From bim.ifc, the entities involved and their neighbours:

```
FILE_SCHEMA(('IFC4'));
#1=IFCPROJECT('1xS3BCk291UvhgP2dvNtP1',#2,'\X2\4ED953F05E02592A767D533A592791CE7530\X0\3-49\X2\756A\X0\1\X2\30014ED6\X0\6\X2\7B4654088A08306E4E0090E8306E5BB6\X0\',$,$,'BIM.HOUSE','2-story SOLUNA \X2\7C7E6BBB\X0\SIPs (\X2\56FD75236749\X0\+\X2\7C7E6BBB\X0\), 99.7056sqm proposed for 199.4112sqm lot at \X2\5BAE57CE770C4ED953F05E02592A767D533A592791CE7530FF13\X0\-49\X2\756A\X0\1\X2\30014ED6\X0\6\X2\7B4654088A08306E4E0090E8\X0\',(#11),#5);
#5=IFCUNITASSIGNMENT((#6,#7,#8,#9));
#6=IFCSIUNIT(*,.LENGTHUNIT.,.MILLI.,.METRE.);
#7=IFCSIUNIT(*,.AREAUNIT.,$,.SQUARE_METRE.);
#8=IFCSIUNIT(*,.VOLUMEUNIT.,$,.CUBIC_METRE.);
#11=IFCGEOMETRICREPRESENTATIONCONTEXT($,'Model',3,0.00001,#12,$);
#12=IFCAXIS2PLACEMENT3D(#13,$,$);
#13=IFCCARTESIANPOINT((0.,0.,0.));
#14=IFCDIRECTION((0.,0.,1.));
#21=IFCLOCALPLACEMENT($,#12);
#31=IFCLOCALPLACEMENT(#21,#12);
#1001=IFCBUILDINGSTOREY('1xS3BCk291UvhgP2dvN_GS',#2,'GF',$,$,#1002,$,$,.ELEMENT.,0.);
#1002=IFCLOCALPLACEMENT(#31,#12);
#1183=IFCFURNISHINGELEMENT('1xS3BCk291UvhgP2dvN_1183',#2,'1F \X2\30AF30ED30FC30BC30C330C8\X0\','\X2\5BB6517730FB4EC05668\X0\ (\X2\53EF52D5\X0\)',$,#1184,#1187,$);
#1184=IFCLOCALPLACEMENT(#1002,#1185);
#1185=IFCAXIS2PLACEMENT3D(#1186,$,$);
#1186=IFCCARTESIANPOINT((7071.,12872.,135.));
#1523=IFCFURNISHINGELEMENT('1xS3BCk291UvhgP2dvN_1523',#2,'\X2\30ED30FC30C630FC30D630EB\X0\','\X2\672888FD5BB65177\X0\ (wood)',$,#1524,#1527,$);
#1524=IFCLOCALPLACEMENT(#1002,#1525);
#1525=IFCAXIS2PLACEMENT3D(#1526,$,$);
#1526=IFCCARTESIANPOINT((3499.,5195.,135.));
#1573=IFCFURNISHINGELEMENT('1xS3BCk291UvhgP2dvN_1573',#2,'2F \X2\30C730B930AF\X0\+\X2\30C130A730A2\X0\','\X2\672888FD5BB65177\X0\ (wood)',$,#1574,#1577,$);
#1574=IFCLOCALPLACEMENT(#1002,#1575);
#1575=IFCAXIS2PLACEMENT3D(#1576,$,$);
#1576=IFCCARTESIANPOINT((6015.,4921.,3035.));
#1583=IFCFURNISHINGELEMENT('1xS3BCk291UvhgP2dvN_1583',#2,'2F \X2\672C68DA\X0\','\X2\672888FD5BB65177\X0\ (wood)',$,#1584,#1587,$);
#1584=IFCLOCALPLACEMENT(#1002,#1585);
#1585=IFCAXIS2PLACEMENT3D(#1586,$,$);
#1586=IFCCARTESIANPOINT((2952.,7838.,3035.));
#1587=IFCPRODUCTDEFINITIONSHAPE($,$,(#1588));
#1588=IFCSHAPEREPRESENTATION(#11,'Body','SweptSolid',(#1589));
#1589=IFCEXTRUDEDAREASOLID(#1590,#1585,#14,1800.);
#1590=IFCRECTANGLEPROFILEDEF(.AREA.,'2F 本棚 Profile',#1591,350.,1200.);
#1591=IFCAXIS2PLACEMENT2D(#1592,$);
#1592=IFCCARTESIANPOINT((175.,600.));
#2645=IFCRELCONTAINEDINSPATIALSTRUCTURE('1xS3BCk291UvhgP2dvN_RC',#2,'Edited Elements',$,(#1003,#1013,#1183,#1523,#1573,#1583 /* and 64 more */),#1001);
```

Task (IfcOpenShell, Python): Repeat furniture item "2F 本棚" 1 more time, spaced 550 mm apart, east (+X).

```python
import numpy as np
import ifcopenshell
import ifcopenshell.api.geometry
import ifcopenshell.api.root
import ifcopenshell.util.element
import ifcopenshell.util.placement

model = ifcopenshell.open("bim.ifc")


def reuse_history(source, copy):
    """copy_class also copies each property set's owner history, people and application; keep the originals."""
    for rel in copy.IsDefinedBy:
        if rel.is_a("IfcRelDefinesByProperties") and (history := rel.RelatingPropertyDefinition.OwnerHistory):
            rel.RelatingPropertyDefinition.OwnerHistory = source.OwnerHistory
            ifcopenshell.util.element.remove_deep2(model, history)


source = model.by_guid("1xS3BCk291UvhgP2dvN_1583")
base = ifcopenshell.util.placement.get_local_placement(source.ObjectPlacement)
step = np.array([1.0, 0.0, 0.0]) * 550.0

for i in range(1, 2):
    copy = ifcopenshell.api.root.copy_class(model, product=source)
    copy.Representation = ifcopenshell.util.element.copy_deep(
        model, source.Representation, exclude=["IfcGeometricRepresentationContext", "IfcRepresentationMap"]
    )
    reuse_history(source, copy)
    matrix = base.copy()
    matrix[:3, 3] += i * step
    print("added at", matrix[:3, 3].round(3) + 0.0)
    ifcopenshell.api.geometry.edit_object_placement(model, product=copy, matrix=matrix, is_si=False)

model.write("bim_rev.ifc")
```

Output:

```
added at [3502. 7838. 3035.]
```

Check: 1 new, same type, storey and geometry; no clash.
